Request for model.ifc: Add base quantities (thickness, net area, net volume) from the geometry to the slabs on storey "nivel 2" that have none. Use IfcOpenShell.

First a look at what the model holds.

```python
import ifcopenshell
import ifcopenshell.util.element
import ifcopenshell.util.unit

model = ifcopenshell.open("model.ifc")
print(model.schema)
for unit_type in ("LENGTHUNIT", "AREAUNIT", "VOLUMEUNIT"):
    print(unit_type, ifcopenshell.util.unit.calculate_unit_scale(model, unit_type))
storey = next(s for s in model.by_type("IfcBuildingStorey") if s.Name == "nivel 2")
slabs = [e for e in ifcopenshell.util.element.get_decomposition(storey) if e.is_a("IfcSlab")]
for e in sorted(slabs, key=lambda e: e.id()):
    print(e.id(), e.is_a(), e.Name, list(ifcopenshell.util.element.get_psets(e, qtos_only=True)), sep=" | ")
```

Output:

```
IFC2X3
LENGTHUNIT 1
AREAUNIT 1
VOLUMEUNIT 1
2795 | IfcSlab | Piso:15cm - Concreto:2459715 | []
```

```python
import ifcopenshell
import ifcopenshell.api.pset
import ifcopenshell.geom
import ifcopenshell.util.element
import ifcopenshell.util.shape
import ifcopenshell.util.unit

model = ifcopenshell.open("model.ifc")
unit_scale = ifcopenshell.util.unit.calculate_unit_scale(model)
area_scale = ifcopenshell.util.unit.calculate_unit_scale(model, "AREAUNIT")
volume_scale = ifcopenshell.util.unit.calculate_unit_scale(model, "VOLUMEUNIT")
settings = ifcopenshell.geom.settings()

storey = next(s for s in model.by_type("IfcBuildingStorey") if s.Name == "nivel 2")
slabs = [e for e in ifcopenshell.util.element.get_decomposition(storey) if e.is_a("IfcSlab")]

for e in sorted(slabs, key=lambda e: e.id()):
    if ifcopenshell.util.element.get_psets(e, qtos_only=True, should_inherit=False):
        continue
    # Geometry comes back in metres, in the element's own axes.
    shape = ifcopenshell.geom.create_shape(settings, e)
    values = {
        "Width": ifcopenshell.util.shape.get_z(shape.geometry) / unit_scale,
        "NetArea": ifcopenshell.util.shape.get_footprint_area(shape.geometry) / area_scale,
        "NetVolume": ifcopenshell.util.shape.get_volume(shape.geometry) / volume_scale,
    }
    qto = ifcopenshell.api.pset.add_qto(model, product=e, name="BaseQuantities")
    ifcopenshell.api.pset.edit_qto(model, qto=qto, properties=values)
    print(e.id(), {k: round(v, 3) for k, v in values.items()})

model.write("model_rev.ifc")
```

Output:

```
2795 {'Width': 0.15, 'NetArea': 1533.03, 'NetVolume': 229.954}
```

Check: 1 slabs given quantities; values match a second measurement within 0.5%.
